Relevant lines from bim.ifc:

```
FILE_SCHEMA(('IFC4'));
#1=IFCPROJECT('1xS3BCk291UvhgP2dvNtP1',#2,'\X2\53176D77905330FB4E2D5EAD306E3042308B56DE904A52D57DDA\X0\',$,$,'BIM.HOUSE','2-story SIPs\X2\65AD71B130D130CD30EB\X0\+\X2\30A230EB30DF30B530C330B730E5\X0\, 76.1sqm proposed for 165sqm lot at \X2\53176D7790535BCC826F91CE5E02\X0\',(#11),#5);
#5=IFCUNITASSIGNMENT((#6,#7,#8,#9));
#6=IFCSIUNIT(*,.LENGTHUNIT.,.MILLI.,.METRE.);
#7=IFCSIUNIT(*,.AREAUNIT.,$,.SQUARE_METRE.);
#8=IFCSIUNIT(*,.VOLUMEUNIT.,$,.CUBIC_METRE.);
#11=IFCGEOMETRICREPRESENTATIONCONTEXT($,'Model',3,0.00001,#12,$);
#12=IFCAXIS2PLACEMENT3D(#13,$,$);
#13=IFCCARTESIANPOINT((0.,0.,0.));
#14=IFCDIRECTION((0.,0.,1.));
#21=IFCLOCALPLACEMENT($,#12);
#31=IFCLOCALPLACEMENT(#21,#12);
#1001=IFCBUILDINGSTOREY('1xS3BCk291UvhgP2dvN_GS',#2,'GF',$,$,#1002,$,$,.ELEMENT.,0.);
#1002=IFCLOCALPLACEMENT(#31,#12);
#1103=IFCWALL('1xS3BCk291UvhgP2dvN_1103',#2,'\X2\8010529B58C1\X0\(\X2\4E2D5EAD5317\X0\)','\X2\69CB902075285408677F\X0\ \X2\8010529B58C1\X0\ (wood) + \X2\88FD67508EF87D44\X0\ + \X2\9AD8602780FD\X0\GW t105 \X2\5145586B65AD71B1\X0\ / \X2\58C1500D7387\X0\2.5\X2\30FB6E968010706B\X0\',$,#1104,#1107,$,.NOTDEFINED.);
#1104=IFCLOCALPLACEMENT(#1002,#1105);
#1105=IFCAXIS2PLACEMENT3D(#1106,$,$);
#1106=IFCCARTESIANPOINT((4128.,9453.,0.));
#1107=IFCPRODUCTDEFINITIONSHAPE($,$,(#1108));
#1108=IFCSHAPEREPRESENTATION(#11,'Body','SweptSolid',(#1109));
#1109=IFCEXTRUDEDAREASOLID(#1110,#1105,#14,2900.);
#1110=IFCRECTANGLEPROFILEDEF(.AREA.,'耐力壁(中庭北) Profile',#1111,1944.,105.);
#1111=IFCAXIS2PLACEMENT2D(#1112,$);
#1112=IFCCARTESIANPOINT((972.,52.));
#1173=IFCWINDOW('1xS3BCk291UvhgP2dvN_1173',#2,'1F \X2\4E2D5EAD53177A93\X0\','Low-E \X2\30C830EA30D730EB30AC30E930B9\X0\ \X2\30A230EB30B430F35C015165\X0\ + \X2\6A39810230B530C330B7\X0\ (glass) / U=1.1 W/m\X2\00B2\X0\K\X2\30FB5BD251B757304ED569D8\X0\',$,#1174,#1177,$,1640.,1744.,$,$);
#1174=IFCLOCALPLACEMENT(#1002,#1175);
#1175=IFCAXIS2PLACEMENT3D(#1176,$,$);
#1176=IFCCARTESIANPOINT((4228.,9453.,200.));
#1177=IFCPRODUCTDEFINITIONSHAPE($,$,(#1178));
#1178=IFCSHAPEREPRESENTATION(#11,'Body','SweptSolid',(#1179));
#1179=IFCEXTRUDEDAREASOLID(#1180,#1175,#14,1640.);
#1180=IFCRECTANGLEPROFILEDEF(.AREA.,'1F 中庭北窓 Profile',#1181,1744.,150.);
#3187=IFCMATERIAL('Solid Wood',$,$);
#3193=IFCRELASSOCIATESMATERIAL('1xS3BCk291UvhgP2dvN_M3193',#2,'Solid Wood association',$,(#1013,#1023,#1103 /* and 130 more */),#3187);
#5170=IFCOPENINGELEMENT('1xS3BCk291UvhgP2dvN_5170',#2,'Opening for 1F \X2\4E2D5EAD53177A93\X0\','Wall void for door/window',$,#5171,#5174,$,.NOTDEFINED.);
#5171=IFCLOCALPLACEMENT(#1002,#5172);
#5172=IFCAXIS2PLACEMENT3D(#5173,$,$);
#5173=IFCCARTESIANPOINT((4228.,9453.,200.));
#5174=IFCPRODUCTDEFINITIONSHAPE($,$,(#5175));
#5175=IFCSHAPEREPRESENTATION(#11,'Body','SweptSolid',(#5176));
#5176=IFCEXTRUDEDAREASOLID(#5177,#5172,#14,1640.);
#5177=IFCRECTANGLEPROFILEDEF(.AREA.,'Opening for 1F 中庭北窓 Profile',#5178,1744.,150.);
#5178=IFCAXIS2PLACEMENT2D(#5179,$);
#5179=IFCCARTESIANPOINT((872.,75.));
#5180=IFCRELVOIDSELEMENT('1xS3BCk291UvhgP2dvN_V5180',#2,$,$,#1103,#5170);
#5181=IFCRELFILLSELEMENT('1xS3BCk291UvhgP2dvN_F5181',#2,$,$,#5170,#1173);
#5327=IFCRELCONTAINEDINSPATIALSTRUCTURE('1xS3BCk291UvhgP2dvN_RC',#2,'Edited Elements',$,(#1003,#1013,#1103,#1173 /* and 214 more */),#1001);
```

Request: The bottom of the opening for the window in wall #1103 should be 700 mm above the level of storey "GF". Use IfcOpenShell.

```python
import numpy as np
import ifcopenshell
import ifcopenshell.api.geometry
import ifcopenshell.geom
import ifcopenshell.util.element
import ifcopenshell.util.placement
import ifcopenshell.util.shape
import ifcopenshell.util.unit

model = ifcopenshell.open("bim.ifc")
unit_scale = ifcopenshell.util.unit.calculate_unit_scale(model)

window = model.by_id(1173)
opening = window.FillsVoids[0].RelatingOpeningElement
storey = ifcopenshell.util.element.get_container(window, ifc_class="IfcBuildingStorey")
level = ifcopenshell.util.placement.get_local_placement(storey.ObjectPlacement)[2, 3]

# The opening's origin need not be at the sill, so measure its lowest point.
shape = ifcopenshell.geom.create_shape(ifcopenshell.geom.settings(), opening)
bottom = ifcopenshell.util.shape.get_shape_bottom_elevation(shape, shape.geometry) / unit_scale
dz = level + 0.7 / unit_scale - bottom

shift = np.array([0.0, 0.0, dz])
# The window is not placed relative to its opening, so move both.
for product in (opening, window):
    matrix = ifcopenshell.util.placement.get_local_placement(product.ObjectPlacement)
    matrix[:3, 3] += shift
    ifcopenshell.api.geometry.edit_object_placement(model, product=product, matrix=matrix, is_si=False)

print(f"moved by {dz * unit_scale:+.3f} m")

model.write("bim_updated.ifc")
```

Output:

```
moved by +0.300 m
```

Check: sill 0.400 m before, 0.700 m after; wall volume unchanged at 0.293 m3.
